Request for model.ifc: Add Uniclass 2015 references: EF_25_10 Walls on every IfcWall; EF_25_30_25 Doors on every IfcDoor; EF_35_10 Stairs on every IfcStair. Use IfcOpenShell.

First a look at what the model holds.

```python
import ifcopenshell

model = ifcopenshell.open("model.ifc")
print(model.schema)
print("classifications:", [c.Name for c in model.by_type("IfcClassification")])
for ifc_class in ("IfcDoor", "IfcRoof", "IfcStair", "IfcWall", "IfcWindow"):
    print(ifc_class, len(model.by_type(ifc_class)))
```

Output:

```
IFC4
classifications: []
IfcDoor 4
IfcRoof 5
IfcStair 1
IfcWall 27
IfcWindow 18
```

```python
import ifcopenshell
import ifcopenshell.api.classification

model = ifcopenshell.open("model.ifc")

system = ifcopenshell.api.classification.add_classification(model, classification="Uniclass 2015")

codes = {
    "IfcWall": ("EF_25_10", "Walls"),
    "IfcDoor": ("EF_25_30_25", "Doors"),
    "IfcStair": ("EF_35_10", "Stairs"),
}
for ifc_class, (code, name) in codes.items():
    products = model.by_type(ifc_class)
    ifcopenshell.api.classification.add_reference(
        model, products=products, classification=system, identification=code, name=name
    )
    print(code, len(products))

model.write("model_edited.ifc")
```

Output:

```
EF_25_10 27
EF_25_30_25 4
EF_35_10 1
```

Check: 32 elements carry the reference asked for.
